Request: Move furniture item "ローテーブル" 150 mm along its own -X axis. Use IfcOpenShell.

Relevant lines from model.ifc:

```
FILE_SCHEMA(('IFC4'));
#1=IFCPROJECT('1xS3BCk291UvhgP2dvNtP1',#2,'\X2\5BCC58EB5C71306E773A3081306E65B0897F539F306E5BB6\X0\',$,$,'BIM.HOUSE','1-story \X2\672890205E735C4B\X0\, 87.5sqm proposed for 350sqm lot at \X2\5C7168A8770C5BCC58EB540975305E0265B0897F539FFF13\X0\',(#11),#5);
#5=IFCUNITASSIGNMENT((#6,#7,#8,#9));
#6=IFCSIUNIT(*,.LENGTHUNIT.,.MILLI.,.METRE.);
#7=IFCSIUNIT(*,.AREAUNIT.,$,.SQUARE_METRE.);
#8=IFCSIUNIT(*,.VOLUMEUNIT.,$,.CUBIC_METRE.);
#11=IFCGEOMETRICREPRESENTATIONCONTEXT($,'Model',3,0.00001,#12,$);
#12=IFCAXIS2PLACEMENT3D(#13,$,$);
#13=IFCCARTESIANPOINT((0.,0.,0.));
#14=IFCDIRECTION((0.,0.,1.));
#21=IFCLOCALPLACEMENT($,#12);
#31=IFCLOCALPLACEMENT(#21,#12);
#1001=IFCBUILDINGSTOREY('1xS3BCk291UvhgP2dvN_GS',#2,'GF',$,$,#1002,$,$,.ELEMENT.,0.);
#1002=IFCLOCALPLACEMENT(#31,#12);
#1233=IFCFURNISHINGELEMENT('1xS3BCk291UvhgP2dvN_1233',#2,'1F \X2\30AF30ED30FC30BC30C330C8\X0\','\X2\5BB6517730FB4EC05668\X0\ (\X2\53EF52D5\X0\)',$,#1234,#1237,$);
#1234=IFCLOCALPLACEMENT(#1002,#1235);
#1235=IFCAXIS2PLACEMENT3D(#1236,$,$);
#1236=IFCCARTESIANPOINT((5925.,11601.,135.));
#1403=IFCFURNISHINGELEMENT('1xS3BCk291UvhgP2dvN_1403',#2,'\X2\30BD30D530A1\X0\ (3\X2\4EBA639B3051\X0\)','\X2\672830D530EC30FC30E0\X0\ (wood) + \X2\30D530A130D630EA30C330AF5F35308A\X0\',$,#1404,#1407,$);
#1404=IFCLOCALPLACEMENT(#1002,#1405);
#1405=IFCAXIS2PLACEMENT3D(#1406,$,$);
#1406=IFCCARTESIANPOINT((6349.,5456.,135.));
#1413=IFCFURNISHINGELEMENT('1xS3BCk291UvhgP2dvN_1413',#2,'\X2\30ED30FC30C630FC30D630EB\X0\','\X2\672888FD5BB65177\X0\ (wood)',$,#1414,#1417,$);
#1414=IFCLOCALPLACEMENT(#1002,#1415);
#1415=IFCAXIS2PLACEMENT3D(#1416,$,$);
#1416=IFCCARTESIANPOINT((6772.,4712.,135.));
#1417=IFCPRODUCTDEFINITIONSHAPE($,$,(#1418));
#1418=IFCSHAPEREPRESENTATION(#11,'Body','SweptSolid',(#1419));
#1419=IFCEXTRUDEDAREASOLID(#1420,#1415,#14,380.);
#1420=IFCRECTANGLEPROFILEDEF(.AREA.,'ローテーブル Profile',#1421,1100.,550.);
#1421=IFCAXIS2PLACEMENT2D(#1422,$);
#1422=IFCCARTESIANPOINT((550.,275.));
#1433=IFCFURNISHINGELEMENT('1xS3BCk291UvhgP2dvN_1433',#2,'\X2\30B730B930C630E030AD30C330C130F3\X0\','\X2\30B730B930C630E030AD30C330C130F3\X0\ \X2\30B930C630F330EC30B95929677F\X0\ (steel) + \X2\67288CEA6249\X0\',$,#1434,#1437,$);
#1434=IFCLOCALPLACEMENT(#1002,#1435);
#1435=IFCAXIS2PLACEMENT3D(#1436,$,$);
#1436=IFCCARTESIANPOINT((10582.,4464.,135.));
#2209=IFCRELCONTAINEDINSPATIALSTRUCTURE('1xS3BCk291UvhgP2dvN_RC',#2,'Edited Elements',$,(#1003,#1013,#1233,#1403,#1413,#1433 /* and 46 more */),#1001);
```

```python
import ifcopenshell
import ifcopenshell.api.geometry
import ifcopenshell.util.placement
import ifcopenshell.util.unit

model = ifcopenshell.open("model.ifc")
unit_scale = ifcopenshell.util.unit.calculate_unit_scale(model)

item = model.by_guid("1xS3BCk291UvhgP2dvN_1413")
matrix = ifcopenshell.util.placement.get_local_placement(item.ObjectPlacement)
matrix[:3, 3] -= matrix[:3, 0] * 0.15 / unit_scale
ifcopenshell.api.geometry.edit_object_placement(model, product=item, matrix=matrix, is_si=False)

print(ifcopenshell.util.placement.get_local_placement(item.ObjectPlacement).round(3) + 0.0)

model.write("model_updated.ifc")
```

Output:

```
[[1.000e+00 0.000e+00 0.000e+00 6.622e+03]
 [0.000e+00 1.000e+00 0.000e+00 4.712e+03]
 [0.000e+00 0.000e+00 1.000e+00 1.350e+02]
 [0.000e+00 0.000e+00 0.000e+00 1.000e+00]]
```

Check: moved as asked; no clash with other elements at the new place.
